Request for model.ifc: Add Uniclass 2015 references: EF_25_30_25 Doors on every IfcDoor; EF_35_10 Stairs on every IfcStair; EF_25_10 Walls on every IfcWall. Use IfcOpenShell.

First a look at what the model holds.

```python
import ifcopenshell

model = ifcopenshell.open("model.ifc")
print(model.schema)
print("classifications:", [c.Name for c in model.by_type("IfcClassification")])
for ifc_class in ("IfcDoor", "IfcRoof", "IfcStair", "IfcWall", "IfcWindow"):
    print(ifc_class, len(model.by_type(ifc_class)))
```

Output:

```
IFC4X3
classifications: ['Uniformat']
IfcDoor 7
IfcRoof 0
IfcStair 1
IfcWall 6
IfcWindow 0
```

```python
import ifcopenshell
import ifcopenshell.api.classification

model = ifcopenshell.open("model.ifc")

system = ifcopenshell.api.classification.add_classification(model, classification="Uniclass 2015")

codes = {
    "IfcDoor": ("EF_25_30_25", "Doors"),
    "IfcStair": ("EF_35_10", "Stairs"),
    "IfcWall": ("EF_25_10", "Walls"),
}
for ifc_class, (code, name) in codes.items():
    products = model.by_type(ifc_class)
    ifcopenshell.api.classification.add_reference(
        model, products=products, classification=system, identification=code, name=name
    )
    print(code, len(products))

model.write("model_edited.ifc")
```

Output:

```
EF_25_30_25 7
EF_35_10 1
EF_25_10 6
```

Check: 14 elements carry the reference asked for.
